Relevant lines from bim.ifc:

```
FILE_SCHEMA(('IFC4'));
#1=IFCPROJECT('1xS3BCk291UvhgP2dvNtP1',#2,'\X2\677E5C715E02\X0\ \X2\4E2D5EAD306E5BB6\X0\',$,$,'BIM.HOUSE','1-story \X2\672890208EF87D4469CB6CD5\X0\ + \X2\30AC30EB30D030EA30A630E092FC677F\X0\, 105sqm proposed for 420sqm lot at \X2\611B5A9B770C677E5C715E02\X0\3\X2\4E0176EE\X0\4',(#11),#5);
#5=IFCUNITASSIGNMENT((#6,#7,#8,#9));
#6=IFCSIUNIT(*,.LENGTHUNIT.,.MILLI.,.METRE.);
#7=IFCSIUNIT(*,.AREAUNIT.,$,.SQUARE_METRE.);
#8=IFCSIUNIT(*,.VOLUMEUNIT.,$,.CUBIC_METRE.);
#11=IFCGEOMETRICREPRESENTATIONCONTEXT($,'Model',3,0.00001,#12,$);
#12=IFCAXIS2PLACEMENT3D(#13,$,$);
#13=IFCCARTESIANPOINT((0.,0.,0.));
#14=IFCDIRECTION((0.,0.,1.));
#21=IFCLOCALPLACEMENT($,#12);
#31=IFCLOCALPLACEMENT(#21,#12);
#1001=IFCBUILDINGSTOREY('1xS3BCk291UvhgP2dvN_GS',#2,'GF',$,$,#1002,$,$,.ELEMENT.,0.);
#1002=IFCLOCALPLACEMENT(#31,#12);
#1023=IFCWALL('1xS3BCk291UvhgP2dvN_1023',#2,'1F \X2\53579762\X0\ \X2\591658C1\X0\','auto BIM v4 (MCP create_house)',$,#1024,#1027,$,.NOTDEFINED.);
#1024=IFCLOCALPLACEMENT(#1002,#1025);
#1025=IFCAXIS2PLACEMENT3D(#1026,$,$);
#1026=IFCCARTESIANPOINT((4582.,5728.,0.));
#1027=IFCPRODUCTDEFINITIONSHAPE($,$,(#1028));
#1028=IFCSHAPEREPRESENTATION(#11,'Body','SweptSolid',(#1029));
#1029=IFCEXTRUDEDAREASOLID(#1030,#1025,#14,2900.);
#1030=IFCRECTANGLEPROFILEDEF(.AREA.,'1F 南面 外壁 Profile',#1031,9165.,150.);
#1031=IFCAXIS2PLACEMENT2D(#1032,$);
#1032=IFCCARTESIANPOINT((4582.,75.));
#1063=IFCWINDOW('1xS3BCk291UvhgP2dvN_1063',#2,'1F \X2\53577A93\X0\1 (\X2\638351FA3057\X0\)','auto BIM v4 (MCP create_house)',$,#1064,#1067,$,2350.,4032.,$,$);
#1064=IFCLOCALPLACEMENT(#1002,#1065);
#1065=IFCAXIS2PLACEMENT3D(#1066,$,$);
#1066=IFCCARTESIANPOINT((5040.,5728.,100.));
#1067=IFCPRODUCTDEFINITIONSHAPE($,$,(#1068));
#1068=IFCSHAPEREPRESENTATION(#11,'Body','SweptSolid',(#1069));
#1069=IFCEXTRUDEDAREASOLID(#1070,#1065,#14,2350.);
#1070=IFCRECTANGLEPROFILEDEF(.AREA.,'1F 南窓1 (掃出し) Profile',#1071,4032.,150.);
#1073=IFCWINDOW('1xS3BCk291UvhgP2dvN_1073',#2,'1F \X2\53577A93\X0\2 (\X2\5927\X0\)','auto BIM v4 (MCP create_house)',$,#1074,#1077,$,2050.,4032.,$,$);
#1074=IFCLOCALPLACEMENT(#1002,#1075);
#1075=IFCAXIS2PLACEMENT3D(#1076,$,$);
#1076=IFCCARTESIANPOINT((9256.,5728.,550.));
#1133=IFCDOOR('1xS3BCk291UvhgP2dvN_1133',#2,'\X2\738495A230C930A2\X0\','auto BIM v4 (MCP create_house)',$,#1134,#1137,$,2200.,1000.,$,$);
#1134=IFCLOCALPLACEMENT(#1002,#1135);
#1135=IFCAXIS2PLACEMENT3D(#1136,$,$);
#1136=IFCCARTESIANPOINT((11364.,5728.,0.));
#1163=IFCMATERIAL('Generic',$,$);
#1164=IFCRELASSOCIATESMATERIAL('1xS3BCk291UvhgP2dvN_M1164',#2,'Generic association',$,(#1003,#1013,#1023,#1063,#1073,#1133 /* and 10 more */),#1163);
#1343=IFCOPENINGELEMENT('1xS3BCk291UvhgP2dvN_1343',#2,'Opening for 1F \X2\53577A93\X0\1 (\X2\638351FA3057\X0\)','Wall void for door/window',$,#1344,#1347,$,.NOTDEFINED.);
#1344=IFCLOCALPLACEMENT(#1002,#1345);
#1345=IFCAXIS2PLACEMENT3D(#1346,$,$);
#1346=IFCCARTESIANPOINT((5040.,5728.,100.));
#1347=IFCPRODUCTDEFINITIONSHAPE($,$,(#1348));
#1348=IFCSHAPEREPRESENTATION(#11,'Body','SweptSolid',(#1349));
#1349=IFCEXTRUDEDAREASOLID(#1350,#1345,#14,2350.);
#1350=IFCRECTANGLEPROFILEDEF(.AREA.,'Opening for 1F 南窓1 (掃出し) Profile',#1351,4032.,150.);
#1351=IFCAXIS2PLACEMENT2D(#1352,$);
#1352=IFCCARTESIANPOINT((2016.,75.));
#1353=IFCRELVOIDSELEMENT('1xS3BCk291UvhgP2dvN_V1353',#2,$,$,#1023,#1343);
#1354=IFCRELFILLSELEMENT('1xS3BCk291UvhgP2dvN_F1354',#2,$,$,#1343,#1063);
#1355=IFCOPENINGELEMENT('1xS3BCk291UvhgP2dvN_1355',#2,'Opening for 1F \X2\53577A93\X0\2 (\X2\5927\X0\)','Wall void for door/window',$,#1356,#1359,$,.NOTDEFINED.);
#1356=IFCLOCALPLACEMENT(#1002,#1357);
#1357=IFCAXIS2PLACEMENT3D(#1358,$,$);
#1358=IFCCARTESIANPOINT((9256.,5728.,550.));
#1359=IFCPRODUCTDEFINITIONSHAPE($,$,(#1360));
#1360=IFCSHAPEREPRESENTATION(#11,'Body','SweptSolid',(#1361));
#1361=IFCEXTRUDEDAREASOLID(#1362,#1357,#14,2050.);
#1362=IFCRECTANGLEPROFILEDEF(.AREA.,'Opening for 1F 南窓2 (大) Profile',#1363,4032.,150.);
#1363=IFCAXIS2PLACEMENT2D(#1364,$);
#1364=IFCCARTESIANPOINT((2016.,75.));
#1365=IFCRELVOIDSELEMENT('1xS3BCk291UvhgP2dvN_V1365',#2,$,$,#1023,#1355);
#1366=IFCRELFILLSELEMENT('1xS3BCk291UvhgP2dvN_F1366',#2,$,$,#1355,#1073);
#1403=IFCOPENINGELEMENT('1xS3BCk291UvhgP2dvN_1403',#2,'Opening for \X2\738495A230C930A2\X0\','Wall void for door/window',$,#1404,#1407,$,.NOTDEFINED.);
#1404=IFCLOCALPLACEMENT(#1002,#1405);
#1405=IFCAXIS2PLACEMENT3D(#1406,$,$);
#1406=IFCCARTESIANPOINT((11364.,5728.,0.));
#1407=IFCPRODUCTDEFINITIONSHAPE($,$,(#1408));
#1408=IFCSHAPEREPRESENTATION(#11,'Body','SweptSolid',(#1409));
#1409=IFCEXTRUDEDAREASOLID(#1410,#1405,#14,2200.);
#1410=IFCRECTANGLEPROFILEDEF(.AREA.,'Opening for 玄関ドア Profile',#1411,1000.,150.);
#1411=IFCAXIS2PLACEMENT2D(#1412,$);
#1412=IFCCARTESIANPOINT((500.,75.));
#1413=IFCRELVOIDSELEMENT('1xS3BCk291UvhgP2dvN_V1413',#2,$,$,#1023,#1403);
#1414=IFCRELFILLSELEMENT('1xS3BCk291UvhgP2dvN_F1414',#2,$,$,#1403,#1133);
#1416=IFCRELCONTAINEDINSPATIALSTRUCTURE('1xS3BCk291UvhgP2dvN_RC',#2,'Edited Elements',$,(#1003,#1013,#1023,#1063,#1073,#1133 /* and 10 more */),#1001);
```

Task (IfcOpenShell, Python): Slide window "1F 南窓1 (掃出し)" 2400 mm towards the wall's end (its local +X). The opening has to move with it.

```python
import ifcopenshell
import ifcopenshell.api.geometry
import ifcopenshell.util.placement
import ifcopenshell.util.unit

model = ifcopenshell.open("bim.ifc")
unit_scale = ifcopenshell.util.unit.calculate_unit_scale(model)

window = model.by_guid("1xS3BCk291UvhgP2dvN_1063")
opening = window.FillsVoids[0].RelatingOpeningElement
wall = opening.VoidsElements[0].RelatingBuildingElement

wall_matrix = ifcopenshell.util.placement.get_local_placement(wall.ObjectPlacement)
shift = wall_matrix[:3, 0] * 2.4 / unit_scale
before = ifcopenshell.util.placement.get_local_placement(window.ObjectPlacement)[:3, 3].copy()

# The window is not placed relative to its opening, so move both.
for product in (opening, window):
    matrix = ifcopenshell.util.placement.get_local_placement(product.ObjectPlacement)
    matrix[:3, 3] += shift
    ifcopenshell.api.geometry.edit_object_placement(model, product=product, matrix=matrix, is_si=False)

after = ifcopenshell.util.placement.get_local_placement(window.ObjectPlacement)[:3, 3]
print("window moved by", (after - before).round(3) + 0.0)

model.write("bim_v2.ifc")
```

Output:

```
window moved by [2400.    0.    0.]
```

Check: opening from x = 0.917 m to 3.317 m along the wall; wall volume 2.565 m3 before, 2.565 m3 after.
